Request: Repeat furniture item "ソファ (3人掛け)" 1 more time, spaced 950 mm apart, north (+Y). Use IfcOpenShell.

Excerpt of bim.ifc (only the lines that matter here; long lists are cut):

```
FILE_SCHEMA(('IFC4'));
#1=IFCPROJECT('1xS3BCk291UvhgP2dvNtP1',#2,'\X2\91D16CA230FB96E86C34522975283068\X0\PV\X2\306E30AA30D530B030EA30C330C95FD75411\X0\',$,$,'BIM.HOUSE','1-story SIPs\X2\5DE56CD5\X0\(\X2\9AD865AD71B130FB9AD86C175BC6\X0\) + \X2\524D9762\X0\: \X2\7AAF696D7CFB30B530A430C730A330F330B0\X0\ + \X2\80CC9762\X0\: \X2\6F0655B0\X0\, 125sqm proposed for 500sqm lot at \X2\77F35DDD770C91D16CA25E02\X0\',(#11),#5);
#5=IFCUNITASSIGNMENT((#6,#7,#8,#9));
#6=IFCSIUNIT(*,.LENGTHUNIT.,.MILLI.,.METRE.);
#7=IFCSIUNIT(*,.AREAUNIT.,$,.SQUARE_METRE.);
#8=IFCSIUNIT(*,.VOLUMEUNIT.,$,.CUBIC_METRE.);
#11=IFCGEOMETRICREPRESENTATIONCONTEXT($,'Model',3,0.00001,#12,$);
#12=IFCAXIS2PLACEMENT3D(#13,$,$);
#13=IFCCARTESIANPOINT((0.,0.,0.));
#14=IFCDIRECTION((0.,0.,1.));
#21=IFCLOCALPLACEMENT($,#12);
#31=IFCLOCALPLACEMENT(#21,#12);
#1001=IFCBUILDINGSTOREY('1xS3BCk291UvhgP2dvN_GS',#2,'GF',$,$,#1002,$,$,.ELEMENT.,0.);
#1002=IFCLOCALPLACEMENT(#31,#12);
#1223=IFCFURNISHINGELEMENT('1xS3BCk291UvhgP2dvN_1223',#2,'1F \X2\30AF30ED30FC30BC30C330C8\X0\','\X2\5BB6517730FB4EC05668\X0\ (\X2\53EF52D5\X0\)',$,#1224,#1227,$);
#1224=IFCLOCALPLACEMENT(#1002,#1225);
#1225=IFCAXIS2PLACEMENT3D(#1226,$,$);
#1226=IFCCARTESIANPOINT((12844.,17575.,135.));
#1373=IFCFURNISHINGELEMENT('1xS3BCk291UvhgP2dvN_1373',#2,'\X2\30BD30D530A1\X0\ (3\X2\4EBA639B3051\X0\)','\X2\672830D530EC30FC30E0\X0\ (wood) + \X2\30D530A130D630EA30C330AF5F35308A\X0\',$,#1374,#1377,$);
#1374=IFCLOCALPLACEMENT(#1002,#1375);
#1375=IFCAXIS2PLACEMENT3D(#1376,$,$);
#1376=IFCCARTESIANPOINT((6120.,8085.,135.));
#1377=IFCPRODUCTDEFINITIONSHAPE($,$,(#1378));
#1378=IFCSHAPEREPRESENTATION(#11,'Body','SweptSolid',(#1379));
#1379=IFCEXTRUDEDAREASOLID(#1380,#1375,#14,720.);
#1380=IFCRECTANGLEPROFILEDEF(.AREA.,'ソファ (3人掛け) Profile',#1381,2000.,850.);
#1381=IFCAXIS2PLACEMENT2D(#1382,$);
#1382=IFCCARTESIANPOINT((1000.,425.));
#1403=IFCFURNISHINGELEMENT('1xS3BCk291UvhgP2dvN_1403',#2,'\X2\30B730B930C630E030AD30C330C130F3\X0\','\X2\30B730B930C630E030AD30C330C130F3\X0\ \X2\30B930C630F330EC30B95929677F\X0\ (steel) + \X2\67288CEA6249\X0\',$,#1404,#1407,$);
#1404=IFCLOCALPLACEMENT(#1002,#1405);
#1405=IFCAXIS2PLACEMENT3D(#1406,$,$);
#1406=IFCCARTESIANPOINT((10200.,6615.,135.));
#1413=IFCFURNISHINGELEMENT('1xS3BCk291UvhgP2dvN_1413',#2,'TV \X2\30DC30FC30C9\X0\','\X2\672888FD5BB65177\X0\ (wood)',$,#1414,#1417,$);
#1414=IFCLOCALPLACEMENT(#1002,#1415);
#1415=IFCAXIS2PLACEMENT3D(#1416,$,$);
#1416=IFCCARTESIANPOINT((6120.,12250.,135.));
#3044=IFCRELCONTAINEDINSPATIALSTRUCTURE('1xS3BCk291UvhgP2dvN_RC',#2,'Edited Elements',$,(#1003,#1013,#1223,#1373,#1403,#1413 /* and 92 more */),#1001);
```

```python
import numpy as np
import ifcopenshell
import ifcopenshell.api.geometry
import ifcopenshell.api.root
import ifcopenshell.util.element
import ifcopenshell.util.placement

model = ifcopenshell.open("bim.ifc")


def reuse_history(source, copy):
    """copy_class also copies each property set's owner history, people and application; keep the originals."""
    for rel in copy.IsDefinedBy:
        if rel.is_a("IfcRelDefinesByProperties") and (history := rel.RelatingPropertyDefinition.OwnerHistory):
            rel.RelatingPropertyDefinition.OwnerHistory = source.OwnerHistory
            ifcopenshell.util.element.remove_deep2(model, history)


source = model.by_id(1373)
base = ifcopenshell.util.placement.get_local_placement(source.ObjectPlacement)
step = np.array([0.0, 1.0, 0.0]) * 950.0

for i in range(1, 2):
    copy = ifcopenshell.api.root.copy_class(model, product=source)
    copy.Representation = ifcopenshell.util.element.copy_deep(
        model, source.Representation, exclude=["IfcGeometricRepresentationContext", "IfcRepresentationMap"]
    )
    reuse_history(source, copy)
    matrix = base.copy()
    matrix[:3, 3] += i * step
    print("added at", matrix[:3, 3].round(3) + 0.0)
    ifcopenshell.api.geometry.edit_object_placement(model, product=copy, matrix=matrix, is_si=False)

model.write("bim_edited.ifc")
```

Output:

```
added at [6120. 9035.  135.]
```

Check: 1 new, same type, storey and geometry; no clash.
